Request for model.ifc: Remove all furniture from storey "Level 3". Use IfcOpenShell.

First a look at what the model holds.

```python
import ifcopenshell
import ifcopenshell.util.element

model = ifcopenshell.open("model.ifc")
print(model.schema)
storey = next(s for s in model.by_type("IfcBuildingStorey") if s.Name == "Level 3")
furniture = [e for e in ifcopenshell.util.element.get_decomposition(storey) if e.is_a("IfcFurnishingElement")]
seen = {}
for e in furniture:
    element_type = ifcopenshell.util.element.get_type(e)
    name = element_type.Name if element_type not in (None, e) else None
    seen[name] = seen.get(name, 0) + 1
for name, count in sorted(seen.items(), key=str):
    print(count, "x", name)
```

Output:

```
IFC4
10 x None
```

```python
import ifcopenshell
import ifcopenshell.api.root
import ifcopenshell.util.element

model = ifcopenshell.open("model.ifc")

storey = next(s for s in model.by_type("IfcBuildingStorey") if s.Name == "Level 3")
furniture = [e for e in ifcopenshell.util.element.get_decomposition(storey) if e.is_a("IfcFurnishingElement")]

for e in furniture:
    ifcopenshell.api.root.remove_product(model, product=e)
print(len(furniture), "removed")

model.write("model_updated.ifc")
```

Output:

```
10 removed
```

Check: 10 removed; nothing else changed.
